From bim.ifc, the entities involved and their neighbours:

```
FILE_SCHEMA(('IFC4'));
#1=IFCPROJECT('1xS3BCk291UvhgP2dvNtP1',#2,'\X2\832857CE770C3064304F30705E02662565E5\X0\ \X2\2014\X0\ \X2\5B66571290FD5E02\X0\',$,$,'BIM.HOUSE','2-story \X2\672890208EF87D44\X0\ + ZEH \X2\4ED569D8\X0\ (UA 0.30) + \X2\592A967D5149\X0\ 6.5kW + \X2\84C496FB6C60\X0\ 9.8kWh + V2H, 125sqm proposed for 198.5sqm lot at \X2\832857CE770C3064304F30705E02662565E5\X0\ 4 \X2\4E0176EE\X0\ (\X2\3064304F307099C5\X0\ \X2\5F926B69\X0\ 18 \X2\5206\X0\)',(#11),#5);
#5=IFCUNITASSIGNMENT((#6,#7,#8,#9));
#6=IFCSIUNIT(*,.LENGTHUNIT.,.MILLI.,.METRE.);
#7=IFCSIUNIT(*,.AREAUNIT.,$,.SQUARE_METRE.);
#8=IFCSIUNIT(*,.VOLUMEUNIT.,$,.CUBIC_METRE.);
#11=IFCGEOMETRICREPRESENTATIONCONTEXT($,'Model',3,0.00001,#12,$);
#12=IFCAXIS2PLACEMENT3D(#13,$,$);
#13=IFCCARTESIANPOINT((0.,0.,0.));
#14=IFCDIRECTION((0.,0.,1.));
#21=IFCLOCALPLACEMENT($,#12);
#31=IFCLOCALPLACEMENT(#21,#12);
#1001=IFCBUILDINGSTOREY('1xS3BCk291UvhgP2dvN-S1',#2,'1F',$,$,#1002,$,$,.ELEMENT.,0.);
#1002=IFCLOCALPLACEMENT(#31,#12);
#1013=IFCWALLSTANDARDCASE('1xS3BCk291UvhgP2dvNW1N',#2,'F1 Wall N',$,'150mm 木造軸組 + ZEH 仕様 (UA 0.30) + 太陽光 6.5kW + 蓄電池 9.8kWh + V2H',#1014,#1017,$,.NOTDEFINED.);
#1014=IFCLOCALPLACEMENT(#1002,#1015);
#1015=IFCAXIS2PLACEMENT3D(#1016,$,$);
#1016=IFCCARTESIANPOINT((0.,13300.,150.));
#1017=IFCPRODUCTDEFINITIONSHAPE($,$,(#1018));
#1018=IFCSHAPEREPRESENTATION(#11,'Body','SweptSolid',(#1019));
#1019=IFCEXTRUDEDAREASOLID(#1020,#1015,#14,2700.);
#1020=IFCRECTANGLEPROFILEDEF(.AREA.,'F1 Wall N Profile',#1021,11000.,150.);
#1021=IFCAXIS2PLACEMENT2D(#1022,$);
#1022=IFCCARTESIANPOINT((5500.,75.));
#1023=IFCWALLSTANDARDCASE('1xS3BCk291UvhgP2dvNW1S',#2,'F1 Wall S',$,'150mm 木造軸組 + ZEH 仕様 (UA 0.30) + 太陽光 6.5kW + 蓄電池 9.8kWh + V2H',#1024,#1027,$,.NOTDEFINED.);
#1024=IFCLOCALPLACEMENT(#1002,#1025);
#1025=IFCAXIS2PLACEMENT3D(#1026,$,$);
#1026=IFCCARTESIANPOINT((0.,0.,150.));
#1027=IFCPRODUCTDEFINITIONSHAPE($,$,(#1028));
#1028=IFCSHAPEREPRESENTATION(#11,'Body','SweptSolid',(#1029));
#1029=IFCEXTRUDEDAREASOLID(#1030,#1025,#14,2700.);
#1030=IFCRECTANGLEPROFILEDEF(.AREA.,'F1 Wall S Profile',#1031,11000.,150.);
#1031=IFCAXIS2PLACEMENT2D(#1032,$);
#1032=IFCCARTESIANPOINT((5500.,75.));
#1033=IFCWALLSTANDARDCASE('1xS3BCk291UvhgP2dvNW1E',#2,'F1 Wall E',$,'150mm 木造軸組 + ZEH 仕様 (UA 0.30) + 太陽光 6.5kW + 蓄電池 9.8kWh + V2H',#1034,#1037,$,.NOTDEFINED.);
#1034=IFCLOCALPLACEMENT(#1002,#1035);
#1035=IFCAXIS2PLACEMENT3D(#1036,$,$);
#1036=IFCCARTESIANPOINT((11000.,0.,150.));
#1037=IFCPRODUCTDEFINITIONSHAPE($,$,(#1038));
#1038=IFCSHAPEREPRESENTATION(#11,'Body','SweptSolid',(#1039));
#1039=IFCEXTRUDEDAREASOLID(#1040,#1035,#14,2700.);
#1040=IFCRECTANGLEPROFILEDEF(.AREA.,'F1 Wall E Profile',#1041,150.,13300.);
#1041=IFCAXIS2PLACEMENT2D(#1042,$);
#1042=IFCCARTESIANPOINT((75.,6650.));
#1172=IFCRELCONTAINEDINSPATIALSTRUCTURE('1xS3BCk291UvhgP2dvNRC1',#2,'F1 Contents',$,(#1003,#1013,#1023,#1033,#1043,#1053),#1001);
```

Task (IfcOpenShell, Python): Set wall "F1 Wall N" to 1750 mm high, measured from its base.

```python
import ifcopenshell
import ifcopenshell.geom
import ifcopenshell.util.shape
import ifcopenshell.util.unit

model = ifcopenshell.open("bim.ifc")
unit_scale = ifcopenshell.util.unit.calculate_unit_scale(model)
settings = ifcopenshell.geom.settings()


def volume(element):
    """Net volume in cubic metres, openings subtracted."""
    shape = ifcopenshell.geom.create_shape(settings, element)
    return ifcopenshell.util.shape.get_volume(shape.geometry)


wall = model.by_id(1013)
before = volume(wall)

body = next(r for r in wall.Representation.Representations if r.RepresentationIdentifier == "Body")
solid = body.Items[0]
old_height = solid.Depth
solid.Depth = 1.75 / unit_scale
after = volume(wall)

print(f"height {old_height:g} -> {solid.Depth:g}, volume {before:.3f} -> {after:.3f} m3")

model.write("bim-out.ifc")
```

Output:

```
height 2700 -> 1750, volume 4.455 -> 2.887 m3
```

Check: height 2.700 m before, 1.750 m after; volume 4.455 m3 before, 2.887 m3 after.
